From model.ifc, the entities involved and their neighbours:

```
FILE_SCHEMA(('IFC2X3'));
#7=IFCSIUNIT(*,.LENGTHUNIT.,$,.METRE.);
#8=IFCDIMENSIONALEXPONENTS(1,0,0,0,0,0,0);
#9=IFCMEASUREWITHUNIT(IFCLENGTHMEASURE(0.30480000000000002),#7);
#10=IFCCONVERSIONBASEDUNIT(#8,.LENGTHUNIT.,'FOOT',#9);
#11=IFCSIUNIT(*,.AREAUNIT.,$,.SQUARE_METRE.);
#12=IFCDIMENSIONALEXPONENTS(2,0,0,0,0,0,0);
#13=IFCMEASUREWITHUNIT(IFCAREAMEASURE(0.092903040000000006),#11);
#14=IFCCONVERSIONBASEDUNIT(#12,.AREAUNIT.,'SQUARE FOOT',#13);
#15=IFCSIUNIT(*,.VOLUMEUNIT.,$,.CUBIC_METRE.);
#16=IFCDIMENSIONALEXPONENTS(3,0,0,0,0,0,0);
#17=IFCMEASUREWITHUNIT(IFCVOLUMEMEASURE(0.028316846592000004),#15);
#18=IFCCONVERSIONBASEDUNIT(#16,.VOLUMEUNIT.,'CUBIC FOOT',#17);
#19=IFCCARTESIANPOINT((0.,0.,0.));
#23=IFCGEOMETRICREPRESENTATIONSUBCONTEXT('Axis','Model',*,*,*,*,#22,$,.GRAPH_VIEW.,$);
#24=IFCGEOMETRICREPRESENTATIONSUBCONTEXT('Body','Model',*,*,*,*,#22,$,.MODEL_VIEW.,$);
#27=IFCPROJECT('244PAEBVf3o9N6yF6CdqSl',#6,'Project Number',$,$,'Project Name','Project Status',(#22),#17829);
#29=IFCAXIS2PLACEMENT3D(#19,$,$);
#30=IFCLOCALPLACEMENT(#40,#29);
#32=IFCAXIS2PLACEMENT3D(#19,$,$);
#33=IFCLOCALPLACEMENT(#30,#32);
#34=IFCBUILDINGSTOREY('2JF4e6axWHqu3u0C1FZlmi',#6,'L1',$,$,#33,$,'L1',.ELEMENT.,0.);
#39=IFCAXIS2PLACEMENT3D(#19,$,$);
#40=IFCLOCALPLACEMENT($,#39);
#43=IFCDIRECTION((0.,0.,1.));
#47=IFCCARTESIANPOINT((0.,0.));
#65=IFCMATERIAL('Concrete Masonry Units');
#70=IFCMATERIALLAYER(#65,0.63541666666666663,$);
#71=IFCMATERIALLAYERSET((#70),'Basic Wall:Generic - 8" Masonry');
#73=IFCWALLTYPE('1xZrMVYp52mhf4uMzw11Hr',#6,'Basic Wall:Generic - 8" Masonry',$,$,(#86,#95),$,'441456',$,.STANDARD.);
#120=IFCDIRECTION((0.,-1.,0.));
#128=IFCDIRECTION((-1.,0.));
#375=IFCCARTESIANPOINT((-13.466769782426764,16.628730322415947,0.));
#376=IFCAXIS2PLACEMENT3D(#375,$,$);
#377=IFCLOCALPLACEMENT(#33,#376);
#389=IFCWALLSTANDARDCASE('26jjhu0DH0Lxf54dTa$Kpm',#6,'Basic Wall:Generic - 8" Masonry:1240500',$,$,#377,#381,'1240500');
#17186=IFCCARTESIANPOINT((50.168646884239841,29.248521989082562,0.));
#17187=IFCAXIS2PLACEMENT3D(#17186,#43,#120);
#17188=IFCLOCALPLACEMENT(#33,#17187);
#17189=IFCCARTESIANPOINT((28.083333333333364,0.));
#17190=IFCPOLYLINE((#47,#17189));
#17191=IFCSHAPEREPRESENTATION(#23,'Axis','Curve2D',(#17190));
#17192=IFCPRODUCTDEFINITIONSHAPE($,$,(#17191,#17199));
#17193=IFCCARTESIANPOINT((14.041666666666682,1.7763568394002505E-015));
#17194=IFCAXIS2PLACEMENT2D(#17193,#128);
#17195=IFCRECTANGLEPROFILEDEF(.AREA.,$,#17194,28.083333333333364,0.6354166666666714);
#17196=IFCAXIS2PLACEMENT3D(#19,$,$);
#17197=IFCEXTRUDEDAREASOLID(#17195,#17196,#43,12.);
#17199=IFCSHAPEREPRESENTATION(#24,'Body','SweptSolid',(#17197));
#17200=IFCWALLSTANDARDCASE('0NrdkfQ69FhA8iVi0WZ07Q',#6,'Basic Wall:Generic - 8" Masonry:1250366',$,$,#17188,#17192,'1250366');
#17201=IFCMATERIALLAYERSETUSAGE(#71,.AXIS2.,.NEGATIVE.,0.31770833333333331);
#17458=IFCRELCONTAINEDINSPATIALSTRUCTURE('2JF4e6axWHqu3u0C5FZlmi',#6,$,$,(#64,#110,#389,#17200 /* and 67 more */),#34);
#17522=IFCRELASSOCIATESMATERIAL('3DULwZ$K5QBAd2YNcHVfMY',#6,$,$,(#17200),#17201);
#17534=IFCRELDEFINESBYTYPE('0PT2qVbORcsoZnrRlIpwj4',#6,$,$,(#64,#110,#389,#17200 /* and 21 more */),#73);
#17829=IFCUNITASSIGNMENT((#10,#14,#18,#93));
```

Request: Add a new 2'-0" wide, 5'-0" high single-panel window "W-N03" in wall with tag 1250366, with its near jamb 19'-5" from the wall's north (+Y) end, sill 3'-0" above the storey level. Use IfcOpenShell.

```python
import numpy as np
import ifcopenshell
import ifcopenshell.api.feature
import ifcopenshell.api.geometry
import ifcopenshell.api.root
import ifcopenshell.api.spatial
import ifcopenshell.api.type
import ifcopenshell.geom
import ifcopenshell.util.element
import ifcopenshell.util.placement
import ifcopenshell.util.representation
import ifcopenshell.util.shape
import ifcopenshell.util.unit

model = ifcopenshell.open("model.ifc")
unit_scale = ifcopenshell.util.unit.calculate_unit_scale(model)
settings = ifcopenshell.geom.settings()


def volume(element):
    """Net volume in cubic metres, openings subtracted."""
    shape = ifcopenshell.geom.create_shape(settings, element)
    return ifcopenshell.util.shape.get_volume(shape.geometry)


wall = model.by_guid("0NrdkfQ69FhA8iVi0WZ07Q")
storey = ifcopenshell.util.element.get_container(wall, ifc_class="IfcBuildingStorey")
context = ifcopenshell.util.representation.get_context(model, "Model", "Body", "MODEL_VIEW")
before = volume(wall)

width, height, from_end, sill = 0.6096, 1.524, 5.9182, 0.9144  # metres

# The wall runs along its own X axis, and the end named is its -X end.
wall_shape = ifcopenshell.geom.create_shape(settings, wall)
x, y, z = ifcopenshell.util.shape.get_vertices(wall_shape.geometry).T
start = x.min() + from_end
face, thickness = float(y.min()), float(y.max() - y.min())
wall_matrix = ifcopenshell.util.placement.get_local_placement(wall.ObjectPlacement)
level = ifcopenshell.util.placement.get_local_placement(storey.ObjectPlacement)[2, 3]


def in_wall(x, y):
    """Placement at x, y metres in the wall's axes, at sill height."""
    matrix = wall_matrix.copy()
    matrix[:, 3] = wall_matrix @ np.array([x / unit_scale, y / unit_scale, 0.0, 1.0])
    matrix[2, 3] = level + sill / unit_scale
    return matrix


# Opening: a box that overshoots both wall faces by 50 mm.
opening = ifcopenshell.api.root.create_entity(model, ifc_class="IfcOpeningElement")
box = ifcopenshell.api.geometry.add_wall_representation(
    model, context=context, length=width, height=height, thickness=thickness + 0.1
)
ifcopenshell.api.geometry.assign_representation(model, product=opening, representation=box)
ifcopenshell.api.geometry.edit_object_placement(model, product=opening, matrix=in_wall(start, face - 0.05), is_si=False)
ifcopenshell.api.feature.add_feature(model, feature=opening, element=wall)

window = ifcopenshell.api.root.create_entity(model, ifc_class="IfcWindow", name="W-N03")
window.OverallWidth, window.OverallHeight = width / unit_scale, height / unit_scale
body = ifcopenshell.api.geometry.add_window_representation(
    model,
    context=context,
    overall_width=window.OverallWidth,
    overall_height=window.OverallHeight,
    partition_type="SINGLE_PANEL",
)
ifcopenshell.api.geometry.assign_representation(model, product=window, representation=body)
ifcopenshell.api.spatial.assign_container(model, products=[window], relating_structure=storey)
fills = ifcopenshell.api.feature.add_filling(model, opening=opening, element=window)
fills.OwnerHistory = window.OwnerHistory  # required in IFC2X3

# IFC2X3 keeps the operation on the window style.
style = ifcopenshell.api.root.create_entity(model, ifc_class="IfcWindowStyle", name="W-N03")
style.OperationType, style.ConstructionType = "SINGLE_PANEL", "NOTDEFINED"
style.ParameterTakesPrecedence = style.Sizeable = False
ifcopenshell.api.type.assign_type(model, related_objects=[window], relating_type=style)

# Centre the window in the wall's thickness.
ifcopenshell.api.geometry.edit_object_placement(model, product=window, matrix=in_wall(start, face), is_si=False)
window_shape = ifcopenshell.geom.create_shape(settings, window)
depth = ifcopenshell.util.shape.get_vertices(window_shape.geometry)[:, 1]
offset = face + thickness / 2 - (depth.min() + depth.max()) / 2
ifcopenshell.api.geometry.edit_object_placement(model, product=window, matrix=in_wall(start, offset), is_si=False)

after = volume(wall)

print(f"wall volume {before:.3f} -> {after:.3f} m3")

model.write("model_rev.ifc")
```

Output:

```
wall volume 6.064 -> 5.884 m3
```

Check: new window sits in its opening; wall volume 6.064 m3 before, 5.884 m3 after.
